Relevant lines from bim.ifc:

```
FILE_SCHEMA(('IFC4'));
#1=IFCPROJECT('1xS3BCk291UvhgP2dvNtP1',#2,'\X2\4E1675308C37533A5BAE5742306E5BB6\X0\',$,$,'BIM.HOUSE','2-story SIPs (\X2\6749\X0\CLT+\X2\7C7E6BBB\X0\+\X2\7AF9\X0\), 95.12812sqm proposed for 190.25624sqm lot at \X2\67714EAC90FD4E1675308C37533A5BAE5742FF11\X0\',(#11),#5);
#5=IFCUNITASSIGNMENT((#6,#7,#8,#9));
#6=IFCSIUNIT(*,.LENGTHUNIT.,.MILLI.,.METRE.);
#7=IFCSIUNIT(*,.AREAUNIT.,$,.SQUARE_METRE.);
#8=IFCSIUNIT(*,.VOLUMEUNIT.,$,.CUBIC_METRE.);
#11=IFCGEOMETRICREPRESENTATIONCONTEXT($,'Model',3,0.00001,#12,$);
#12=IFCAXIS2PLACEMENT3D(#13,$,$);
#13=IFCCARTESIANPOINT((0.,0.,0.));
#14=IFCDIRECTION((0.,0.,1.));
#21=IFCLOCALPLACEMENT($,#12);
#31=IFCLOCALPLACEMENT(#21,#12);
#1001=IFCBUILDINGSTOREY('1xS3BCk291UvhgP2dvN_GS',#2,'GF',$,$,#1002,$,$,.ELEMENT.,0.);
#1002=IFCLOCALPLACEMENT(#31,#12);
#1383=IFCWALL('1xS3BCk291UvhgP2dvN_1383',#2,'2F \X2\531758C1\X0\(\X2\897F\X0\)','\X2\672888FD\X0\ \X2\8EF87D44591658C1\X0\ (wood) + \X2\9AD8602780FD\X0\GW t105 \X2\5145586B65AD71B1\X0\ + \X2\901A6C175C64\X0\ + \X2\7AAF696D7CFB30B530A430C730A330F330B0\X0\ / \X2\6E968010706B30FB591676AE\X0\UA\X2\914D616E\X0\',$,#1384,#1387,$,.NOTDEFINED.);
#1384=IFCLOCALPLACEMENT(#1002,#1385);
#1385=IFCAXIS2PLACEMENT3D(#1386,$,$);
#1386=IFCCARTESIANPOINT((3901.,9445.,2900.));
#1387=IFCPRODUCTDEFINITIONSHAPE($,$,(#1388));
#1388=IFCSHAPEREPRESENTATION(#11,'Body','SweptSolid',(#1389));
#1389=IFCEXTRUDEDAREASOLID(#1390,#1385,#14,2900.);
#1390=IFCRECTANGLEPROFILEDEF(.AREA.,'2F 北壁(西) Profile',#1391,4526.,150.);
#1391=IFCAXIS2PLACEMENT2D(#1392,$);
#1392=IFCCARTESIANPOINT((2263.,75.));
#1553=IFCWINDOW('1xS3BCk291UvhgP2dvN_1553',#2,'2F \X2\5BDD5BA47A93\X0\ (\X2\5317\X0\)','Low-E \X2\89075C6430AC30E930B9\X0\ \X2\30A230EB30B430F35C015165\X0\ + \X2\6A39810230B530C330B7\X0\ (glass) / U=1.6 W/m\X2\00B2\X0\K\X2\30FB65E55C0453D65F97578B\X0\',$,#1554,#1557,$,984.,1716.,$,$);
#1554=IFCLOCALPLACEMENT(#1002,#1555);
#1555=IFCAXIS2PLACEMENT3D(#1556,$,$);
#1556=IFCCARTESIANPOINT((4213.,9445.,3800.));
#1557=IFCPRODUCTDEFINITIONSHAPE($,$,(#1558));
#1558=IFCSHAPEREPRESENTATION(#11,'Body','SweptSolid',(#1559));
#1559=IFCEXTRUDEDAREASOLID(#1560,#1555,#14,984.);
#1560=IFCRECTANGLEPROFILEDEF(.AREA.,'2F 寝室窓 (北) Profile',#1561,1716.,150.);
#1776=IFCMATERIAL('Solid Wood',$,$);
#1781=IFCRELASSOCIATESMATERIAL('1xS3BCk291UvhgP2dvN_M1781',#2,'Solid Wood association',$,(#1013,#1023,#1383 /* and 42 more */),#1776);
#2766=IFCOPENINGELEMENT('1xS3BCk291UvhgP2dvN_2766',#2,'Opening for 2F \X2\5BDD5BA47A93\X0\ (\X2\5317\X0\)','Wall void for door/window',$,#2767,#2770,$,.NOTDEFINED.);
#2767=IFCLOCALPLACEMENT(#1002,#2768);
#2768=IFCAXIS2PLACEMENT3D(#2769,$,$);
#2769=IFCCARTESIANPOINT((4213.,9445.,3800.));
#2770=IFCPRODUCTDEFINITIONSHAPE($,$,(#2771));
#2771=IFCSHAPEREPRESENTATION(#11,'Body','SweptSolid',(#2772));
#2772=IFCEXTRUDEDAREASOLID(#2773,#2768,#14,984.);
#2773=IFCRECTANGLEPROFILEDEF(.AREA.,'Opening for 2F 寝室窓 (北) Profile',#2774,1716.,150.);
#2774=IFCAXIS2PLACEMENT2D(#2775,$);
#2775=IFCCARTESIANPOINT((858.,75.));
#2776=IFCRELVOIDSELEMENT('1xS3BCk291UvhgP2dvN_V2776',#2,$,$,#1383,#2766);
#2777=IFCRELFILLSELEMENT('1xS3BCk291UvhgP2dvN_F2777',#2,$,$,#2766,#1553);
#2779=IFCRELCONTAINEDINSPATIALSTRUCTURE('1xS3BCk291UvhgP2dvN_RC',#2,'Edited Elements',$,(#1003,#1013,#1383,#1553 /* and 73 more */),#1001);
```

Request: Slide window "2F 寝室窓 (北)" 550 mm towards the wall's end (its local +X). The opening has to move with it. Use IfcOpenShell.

```python
import ifcopenshell
import ifcopenshell.api.geometry
import ifcopenshell.util.placement
import ifcopenshell.util.unit

model = ifcopenshell.open("bim.ifc")
unit_scale = ifcopenshell.util.unit.calculate_unit_scale(model)

window = model.by_guid("1xS3BCk291UvhgP2dvN_1553")
opening = window.FillsVoids[0].RelatingOpeningElement
wall = opening.VoidsElements[0].RelatingBuildingElement

wall_matrix = ifcopenshell.util.placement.get_local_placement(wall.ObjectPlacement)
shift = wall_matrix[:3, 0] * 0.55 / unit_scale
before = ifcopenshell.util.placement.get_local_placement(window.ObjectPlacement)[:3, 3].copy()

# The window is not placed relative to its opening, so move both.
for product in (opening, window):
    matrix = ifcopenshell.util.placement.get_local_placement(product.ObjectPlacement)
    matrix[:3, 3] += shift
    ifcopenshell.api.geometry.edit_object_placement(model, product=product, matrix=matrix, is_si=False)

after = ifcopenshell.util.placement.get_local_placement(window.ObjectPlacement)[:3, 3]
print("window moved by", (after - before).round(3) + 0.0)

model.write("bim_rev.ifc")
```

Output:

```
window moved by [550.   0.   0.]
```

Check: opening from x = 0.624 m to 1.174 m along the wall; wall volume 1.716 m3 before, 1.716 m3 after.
